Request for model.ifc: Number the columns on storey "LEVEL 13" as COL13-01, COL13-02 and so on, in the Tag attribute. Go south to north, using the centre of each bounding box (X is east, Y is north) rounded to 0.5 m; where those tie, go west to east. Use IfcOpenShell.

First a look at what the model holds.

```python
import ifcopenshell
import ifcopenshell.util.element
import ifcopenshell.util.placement

model = ifcopenshell.open("model.ifc")
print(model.schema)
storey = next(s for s in model.by_type("IfcBuildingStorey") if s.Name == "LEVEL 13")
columns = [e for e in ifcopenshell.util.element.get_decomposition(storey) if e.is_a("IfcColumn")]
for e in sorted(columns, key=lambda e: e.id()):
    origin = ifcopenshell.util.placement.get_local_placement(e.ObjectPlacement)[:3, 3]
    print(e.id(), e.Tag, e.Name, origin.round(2) + 0.0, sep=" | ")
```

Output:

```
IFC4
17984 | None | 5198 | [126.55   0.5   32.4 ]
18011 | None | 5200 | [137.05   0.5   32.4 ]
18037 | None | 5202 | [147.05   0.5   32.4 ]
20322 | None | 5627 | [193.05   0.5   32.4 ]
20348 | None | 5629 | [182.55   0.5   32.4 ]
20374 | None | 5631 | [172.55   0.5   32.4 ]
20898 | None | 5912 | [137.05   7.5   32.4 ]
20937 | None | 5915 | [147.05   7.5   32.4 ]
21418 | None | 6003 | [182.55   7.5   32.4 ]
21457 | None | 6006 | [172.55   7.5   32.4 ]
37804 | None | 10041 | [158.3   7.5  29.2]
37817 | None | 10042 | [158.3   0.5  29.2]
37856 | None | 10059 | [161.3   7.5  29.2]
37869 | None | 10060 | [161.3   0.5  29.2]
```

```python
import ifcopenshell
import ifcopenshell.geom
import ifcopenshell.util.element
import ifcopenshell.util.shape

model = ifcopenshell.open("model.ifc")
settings = ifcopenshell.geom.settings()
settings.set("use-world-coords", True)


def centre(element):
    shape = ifcopenshell.geom.create_shape(settings, element)
    return ifcopenshell.util.shape.get_bbox_centroid(shape.geometry)


storey = next(s for s in model.by_type("IfcBuildingStorey") if s.Name == "LEVEL 13")
columns = [e for e in ifcopenshell.util.element.get_decomposition(storey) if e.is_a("IfcColumn")]

# Insertion points can sit at a corner or the storey origin, so sort by the geometry (in metres).
centres = {e: centre(e) for e in columns}
columns.sort(key=lambda e: (round(centres[e][1] / 0.5), centres[e][0]))

for i, e in enumerate(columns, start=1):
    number = f"COL13-{i:02d}"
    e.Tag = number
    print(e.id(), number)

model.write("model_edited.ifc")
```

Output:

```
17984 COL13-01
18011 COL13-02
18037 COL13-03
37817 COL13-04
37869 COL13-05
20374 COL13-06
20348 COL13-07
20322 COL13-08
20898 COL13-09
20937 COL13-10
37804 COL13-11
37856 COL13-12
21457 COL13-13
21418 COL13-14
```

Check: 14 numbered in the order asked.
